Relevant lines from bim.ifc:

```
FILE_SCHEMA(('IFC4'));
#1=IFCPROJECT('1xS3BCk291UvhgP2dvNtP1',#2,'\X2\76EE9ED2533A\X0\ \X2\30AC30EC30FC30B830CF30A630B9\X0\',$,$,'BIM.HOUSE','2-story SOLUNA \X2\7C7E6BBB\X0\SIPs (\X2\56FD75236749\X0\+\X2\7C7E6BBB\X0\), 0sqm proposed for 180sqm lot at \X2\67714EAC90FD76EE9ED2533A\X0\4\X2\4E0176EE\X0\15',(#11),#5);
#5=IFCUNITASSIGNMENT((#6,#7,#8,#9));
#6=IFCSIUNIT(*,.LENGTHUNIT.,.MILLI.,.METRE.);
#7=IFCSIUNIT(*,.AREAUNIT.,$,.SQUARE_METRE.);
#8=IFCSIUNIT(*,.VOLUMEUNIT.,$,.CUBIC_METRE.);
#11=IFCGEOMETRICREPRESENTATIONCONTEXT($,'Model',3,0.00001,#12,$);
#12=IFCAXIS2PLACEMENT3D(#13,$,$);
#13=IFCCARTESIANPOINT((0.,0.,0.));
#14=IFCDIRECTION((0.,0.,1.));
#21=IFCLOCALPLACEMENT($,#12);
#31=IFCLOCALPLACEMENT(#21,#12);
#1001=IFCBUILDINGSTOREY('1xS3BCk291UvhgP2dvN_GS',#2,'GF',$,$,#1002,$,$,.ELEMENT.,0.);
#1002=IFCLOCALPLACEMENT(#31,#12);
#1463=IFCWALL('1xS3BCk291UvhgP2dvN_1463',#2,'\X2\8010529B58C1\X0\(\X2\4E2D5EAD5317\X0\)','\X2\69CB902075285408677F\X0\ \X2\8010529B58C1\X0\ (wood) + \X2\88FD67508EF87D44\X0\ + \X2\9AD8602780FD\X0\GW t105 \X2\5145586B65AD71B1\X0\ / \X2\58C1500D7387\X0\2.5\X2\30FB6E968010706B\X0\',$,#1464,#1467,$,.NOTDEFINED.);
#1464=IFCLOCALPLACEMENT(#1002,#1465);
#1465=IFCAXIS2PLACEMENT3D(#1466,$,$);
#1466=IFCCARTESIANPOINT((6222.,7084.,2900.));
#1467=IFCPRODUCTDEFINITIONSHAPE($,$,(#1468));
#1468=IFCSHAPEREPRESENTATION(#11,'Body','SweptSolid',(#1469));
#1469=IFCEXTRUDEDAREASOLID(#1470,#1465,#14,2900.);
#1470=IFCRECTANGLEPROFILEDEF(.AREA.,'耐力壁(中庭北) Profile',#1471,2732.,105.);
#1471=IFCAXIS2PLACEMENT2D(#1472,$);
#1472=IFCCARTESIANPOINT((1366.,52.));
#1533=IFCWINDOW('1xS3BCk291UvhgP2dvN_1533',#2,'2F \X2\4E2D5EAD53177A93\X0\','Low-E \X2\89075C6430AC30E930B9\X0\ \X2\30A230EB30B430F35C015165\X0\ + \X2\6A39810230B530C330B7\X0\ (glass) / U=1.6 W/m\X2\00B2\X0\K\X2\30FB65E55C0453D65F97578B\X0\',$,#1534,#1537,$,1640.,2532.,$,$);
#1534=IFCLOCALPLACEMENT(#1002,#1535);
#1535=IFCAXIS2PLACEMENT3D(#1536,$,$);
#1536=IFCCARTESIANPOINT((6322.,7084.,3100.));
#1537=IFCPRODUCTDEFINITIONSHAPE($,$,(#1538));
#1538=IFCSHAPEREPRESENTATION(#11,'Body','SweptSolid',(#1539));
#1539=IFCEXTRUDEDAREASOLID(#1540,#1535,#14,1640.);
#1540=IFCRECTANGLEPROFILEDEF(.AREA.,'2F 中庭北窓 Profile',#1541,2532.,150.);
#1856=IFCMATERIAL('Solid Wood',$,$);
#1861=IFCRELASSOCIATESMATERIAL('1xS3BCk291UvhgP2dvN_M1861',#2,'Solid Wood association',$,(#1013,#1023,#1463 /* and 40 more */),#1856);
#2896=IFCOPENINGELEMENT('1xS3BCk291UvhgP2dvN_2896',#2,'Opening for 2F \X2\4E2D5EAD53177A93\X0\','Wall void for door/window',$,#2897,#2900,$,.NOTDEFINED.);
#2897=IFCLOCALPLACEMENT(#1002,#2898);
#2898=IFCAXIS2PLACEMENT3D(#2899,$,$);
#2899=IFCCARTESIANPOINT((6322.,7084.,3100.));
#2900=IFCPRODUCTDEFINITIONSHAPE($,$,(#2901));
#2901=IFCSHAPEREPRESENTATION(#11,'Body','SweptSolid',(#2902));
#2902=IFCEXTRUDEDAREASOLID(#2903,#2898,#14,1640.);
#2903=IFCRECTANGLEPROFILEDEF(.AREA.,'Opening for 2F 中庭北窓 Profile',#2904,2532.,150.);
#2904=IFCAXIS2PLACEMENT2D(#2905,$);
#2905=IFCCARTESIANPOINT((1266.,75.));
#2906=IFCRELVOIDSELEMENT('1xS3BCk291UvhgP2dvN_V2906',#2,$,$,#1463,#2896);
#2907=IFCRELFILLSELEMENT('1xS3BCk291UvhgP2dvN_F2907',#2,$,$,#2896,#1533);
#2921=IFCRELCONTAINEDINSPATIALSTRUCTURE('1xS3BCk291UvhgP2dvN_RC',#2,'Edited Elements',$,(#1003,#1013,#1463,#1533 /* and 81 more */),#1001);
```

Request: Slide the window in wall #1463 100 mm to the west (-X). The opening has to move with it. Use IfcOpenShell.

```python
import ifcopenshell
import ifcopenshell.api.geometry
import ifcopenshell.util.placement

model = ifcopenshell.open("bim.ifc")

window = model.by_guid("1xS3BCk291UvhgP2dvN_1533")
opening = window.FillsVoids[0].RelatingOpeningElement
wall = opening.VoidsElements[0].RelatingBuildingElement

wall_matrix = ifcopenshell.util.placement.get_local_placement(wall.ObjectPlacement)
shift = wall_matrix[:3, 0] * -100.0
before = ifcopenshell.util.placement.get_local_placement(window.ObjectPlacement)[:3, 3].copy()

# The window is not placed relative to its opening, so move both.
for product in (opening, window):
    matrix = ifcopenshell.util.placement.get_local_placement(product.ObjectPlacement)
    matrix[:3, 3] += shift
    ifcopenshell.api.geometry.edit_object_placement(model, product=product, matrix=matrix, is_si=False)

after = ifcopenshell.util.placement.get_local_placement(window.ObjectPlacement)[:3, 3]
print("window moved by", (after - before).round(3) + 0.0)

model.write("bim-out.ifc")
```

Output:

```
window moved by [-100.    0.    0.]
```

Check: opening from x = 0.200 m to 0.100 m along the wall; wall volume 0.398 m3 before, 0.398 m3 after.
